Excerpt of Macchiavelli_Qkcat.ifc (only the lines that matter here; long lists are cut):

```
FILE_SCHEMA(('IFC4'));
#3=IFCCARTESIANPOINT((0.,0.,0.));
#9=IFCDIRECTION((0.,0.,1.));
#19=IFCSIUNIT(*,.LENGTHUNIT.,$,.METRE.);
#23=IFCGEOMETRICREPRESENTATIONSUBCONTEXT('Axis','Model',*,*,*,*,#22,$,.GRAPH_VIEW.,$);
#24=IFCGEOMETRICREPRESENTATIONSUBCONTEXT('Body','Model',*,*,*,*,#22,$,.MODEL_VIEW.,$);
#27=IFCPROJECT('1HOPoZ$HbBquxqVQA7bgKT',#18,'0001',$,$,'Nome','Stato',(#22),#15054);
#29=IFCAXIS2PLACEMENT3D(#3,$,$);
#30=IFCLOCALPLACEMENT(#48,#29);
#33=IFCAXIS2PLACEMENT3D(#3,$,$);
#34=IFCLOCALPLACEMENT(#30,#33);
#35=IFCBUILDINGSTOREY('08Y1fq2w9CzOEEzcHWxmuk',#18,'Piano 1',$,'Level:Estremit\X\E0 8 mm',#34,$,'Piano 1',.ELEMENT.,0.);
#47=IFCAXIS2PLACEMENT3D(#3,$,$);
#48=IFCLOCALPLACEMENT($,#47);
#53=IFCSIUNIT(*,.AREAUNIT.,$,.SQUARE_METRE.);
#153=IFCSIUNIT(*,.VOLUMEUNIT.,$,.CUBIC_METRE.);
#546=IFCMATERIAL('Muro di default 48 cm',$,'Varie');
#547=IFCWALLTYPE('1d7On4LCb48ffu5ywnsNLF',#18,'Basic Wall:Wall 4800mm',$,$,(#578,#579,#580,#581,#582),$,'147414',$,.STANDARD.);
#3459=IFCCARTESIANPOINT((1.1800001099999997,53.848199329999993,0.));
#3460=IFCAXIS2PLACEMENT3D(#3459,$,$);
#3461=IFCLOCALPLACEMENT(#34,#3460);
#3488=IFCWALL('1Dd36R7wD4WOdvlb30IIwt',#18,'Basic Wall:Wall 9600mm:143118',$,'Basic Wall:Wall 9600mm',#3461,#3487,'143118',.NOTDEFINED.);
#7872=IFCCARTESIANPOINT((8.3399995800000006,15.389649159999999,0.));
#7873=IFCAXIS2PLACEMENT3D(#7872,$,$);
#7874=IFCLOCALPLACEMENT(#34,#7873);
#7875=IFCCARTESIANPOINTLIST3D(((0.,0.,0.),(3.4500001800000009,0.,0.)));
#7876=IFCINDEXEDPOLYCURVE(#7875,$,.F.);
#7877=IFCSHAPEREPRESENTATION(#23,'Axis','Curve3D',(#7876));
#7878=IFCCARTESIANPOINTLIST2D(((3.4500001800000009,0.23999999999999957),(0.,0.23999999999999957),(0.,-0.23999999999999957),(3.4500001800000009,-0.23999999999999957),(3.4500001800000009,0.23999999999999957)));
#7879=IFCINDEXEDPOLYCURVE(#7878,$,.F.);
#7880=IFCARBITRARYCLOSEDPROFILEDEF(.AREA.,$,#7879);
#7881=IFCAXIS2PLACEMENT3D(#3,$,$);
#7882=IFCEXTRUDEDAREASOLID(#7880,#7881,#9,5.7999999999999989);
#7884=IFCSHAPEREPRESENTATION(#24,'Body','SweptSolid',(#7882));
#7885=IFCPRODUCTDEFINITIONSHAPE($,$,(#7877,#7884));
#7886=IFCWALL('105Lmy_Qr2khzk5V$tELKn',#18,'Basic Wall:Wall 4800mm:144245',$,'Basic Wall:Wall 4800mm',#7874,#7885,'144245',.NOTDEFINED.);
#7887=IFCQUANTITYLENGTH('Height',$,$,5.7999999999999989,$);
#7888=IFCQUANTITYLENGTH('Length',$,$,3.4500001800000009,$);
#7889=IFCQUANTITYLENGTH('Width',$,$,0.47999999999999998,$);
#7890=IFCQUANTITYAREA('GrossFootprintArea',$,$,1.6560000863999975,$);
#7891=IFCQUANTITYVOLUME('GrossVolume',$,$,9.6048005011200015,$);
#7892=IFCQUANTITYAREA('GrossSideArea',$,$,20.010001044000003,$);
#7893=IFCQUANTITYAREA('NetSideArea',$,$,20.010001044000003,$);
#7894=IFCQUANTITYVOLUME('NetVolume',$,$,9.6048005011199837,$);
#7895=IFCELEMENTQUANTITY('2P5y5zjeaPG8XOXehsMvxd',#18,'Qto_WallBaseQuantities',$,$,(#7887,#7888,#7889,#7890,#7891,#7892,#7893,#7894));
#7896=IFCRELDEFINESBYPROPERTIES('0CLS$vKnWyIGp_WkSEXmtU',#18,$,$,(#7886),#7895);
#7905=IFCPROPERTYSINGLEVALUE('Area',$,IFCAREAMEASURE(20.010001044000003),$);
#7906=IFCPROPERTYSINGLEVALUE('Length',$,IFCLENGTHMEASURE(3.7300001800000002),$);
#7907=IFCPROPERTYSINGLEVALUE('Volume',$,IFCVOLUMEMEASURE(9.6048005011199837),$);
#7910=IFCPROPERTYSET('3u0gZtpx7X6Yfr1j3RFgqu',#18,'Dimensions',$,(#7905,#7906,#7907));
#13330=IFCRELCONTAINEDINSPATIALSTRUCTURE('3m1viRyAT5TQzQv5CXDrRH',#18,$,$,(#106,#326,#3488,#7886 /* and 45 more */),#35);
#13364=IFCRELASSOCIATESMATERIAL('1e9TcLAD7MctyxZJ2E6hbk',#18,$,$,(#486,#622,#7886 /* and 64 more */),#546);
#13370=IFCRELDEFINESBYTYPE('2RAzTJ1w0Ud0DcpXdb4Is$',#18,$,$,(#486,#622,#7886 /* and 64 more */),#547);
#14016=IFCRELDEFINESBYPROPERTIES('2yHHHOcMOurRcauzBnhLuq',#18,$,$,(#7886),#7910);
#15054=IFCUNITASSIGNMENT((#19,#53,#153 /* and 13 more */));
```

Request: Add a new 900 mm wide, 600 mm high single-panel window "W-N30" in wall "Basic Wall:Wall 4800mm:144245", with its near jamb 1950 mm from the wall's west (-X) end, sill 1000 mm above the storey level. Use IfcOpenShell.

```python
import numpy as np
import ifcopenshell
import ifcopenshell.api.feature
import ifcopenshell.api.geometry
import ifcopenshell.api.pset
import ifcopenshell.api.root
import ifcopenshell.api.spatial
import ifcopenshell.geom
import ifcopenshell.util.element
import ifcopenshell.util.placement
import ifcopenshell.util.representation
import ifcopenshell.util.shape
import ifcopenshell.util.unit

model = ifcopenshell.open("Macchiavelli_Qkcat.ifc")
unit_scale = ifcopenshell.util.unit.calculate_unit_scale(model)
area_scale = ifcopenshell.util.unit.calculate_unit_scale(model, "AREAUNIT")
volume_scale = ifcopenshell.util.unit.calculate_unit_scale(model, "VOLUMEUNIT")
settings = ifcopenshell.geom.settings()


def volume(element):
    """Net volume in cubic metres, openings subtracted."""
    shape = ifcopenshell.geom.create_shape(settings, element)
    return ifcopenshell.util.shape.get_volume(shape.geometry)


wall = model.by_guid("105Lmy_Qr2khzk5V$tELKn")
storey = ifcopenshell.util.element.get_container(wall, ifc_class="IfcBuildingStorey")
context = ifcopenshell.util.representation.get_context(model, "Model", "Body", "MODEL_VIEW")
before = volume(wall)

width, height, from_end, sill = 0.9, 0.6, 1.95, 1  # metres

# The wall runs along its own X axis, and the end named is its -X end.
wall_shape = ifcopenshell.geom.create_shape(settings, wall)
x, y, z = ifcopenshell.util.shape.get_vertices(wall_shape.geometry).T
start = x.min() + from_end
face, thickness = float(y.min()), float(y.max() - y.min())
wall_matrix = ifcopenshell.util.placement.get_local_placement(wall.ObjectPlacement)
level = ifcopenshell.util.placement.get_local_placement(storey.ObjectPlacement)[2, 3]


def in_wall(x, y):
    """Placement at x, y metres in the wall's axes, at sill height."""
    matrix = wall_matrix.copy()
    matrix[:, 3] = wall_matrix @ np.array([x / unit_scale, y / unit_scale, 0.0, 1.0])
    matrix[2, 3] = level + sill / unit_scale
    return matrix


# Opening: a box that overshoots both wall faces by 50 mm.
opening = ifcopenshell.api.root.create_entity(model, ifc_class="IfcOpeningElement", predefined_type="OPENING")
box = ifcopenshell.api.geometry.add_wall_representation(
    model, context=context, length=width, height=height, thickness=thickness + 0.1
)
ifcopenshell.api.geometry.assign_representation(model, product=opening, representation=box)
ifcopenshell.api.geometry.edit_object_placement(model, product=opening, matrix=in_wall(start, face - 0.05), is_si=False)
ifcopenshell.api.feature.add_feature(model, feature=opening, element=wall)

window = ifcopenshell.api.root.create_entity(model, ifc_class="IfcWindow", name="W-N30", predefined_type="WINDOW")
window.OverallWidth, window.OverallHeight = width / unit_scale, height / unit_scale
window.PartitioningType = "SINGLE_PANEL"
body = ifcopenshell.api.geometry.add_window_representation(
    model,
    context=context,
    overall_width=window.OverallWidth,
    overall_height=window.OverallHeight,
    partition_type="SINGLE_PANEL",
)
ifcopenshell.api.geometry.assign_representation(model, product=window, representation=body)
ifcopenshell.api.spatial.assign_container(model, products=[window], relating_structure=storey)
ifcopenshell.api.feature.add_filling(model, opening=opening, element=window)

# Centre the window in the wall's thickness.
ifcopenshell.api.geometry.edit_object_placement(model, product=window, matrix=in_wall(start, face), is_si=False)
window_shape = ifcopenshell.geom.create_shape(settings, window)
depth = ifcopenshell.util.shape.get_vertices(window_shape.geometry)[:, 1]
offset = face + thickness / 2 - (depth.min() + depth.max()) / 2
ifcopenshell.api.geometry.edit_object_placement(model, product=window, matrix=in_wall(start, offset), is_si=False)

after = volume(wall)

# Update the wall's stored quantities.
qto = model.by_id(ifcopenshell.util.element.get_pset(wall, "Qto_WallBaseQuantities", should_inherit=False)["id"])
ifcopenshell.api.pset.edit_qto(model, qto=qto, properties={
    "NetSideArea": after / thickness / area_scale,
    "NetVolume": after / volume_scale,
})
pset = model.by_id(ifcopenshell.util.element.get_pset(wall, "Dimensions", should_inherit=False)["id"])
ifcopenshell.api.pset.edit_pset(model, pset=pset, properties={
    "Area": model.create_entity("IfcAreaMeasure", after / thickness / area_scale),
    "Volume": model.create_entity("IfcVolumeMeasure", after / volume_scale),
})

print(f"wall volume {before:.3f} -> {after:.3f} m3")

model.write("Macchiavelli_Qkcat-out.ifc")
```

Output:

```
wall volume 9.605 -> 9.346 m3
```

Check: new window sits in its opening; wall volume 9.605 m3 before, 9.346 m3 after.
